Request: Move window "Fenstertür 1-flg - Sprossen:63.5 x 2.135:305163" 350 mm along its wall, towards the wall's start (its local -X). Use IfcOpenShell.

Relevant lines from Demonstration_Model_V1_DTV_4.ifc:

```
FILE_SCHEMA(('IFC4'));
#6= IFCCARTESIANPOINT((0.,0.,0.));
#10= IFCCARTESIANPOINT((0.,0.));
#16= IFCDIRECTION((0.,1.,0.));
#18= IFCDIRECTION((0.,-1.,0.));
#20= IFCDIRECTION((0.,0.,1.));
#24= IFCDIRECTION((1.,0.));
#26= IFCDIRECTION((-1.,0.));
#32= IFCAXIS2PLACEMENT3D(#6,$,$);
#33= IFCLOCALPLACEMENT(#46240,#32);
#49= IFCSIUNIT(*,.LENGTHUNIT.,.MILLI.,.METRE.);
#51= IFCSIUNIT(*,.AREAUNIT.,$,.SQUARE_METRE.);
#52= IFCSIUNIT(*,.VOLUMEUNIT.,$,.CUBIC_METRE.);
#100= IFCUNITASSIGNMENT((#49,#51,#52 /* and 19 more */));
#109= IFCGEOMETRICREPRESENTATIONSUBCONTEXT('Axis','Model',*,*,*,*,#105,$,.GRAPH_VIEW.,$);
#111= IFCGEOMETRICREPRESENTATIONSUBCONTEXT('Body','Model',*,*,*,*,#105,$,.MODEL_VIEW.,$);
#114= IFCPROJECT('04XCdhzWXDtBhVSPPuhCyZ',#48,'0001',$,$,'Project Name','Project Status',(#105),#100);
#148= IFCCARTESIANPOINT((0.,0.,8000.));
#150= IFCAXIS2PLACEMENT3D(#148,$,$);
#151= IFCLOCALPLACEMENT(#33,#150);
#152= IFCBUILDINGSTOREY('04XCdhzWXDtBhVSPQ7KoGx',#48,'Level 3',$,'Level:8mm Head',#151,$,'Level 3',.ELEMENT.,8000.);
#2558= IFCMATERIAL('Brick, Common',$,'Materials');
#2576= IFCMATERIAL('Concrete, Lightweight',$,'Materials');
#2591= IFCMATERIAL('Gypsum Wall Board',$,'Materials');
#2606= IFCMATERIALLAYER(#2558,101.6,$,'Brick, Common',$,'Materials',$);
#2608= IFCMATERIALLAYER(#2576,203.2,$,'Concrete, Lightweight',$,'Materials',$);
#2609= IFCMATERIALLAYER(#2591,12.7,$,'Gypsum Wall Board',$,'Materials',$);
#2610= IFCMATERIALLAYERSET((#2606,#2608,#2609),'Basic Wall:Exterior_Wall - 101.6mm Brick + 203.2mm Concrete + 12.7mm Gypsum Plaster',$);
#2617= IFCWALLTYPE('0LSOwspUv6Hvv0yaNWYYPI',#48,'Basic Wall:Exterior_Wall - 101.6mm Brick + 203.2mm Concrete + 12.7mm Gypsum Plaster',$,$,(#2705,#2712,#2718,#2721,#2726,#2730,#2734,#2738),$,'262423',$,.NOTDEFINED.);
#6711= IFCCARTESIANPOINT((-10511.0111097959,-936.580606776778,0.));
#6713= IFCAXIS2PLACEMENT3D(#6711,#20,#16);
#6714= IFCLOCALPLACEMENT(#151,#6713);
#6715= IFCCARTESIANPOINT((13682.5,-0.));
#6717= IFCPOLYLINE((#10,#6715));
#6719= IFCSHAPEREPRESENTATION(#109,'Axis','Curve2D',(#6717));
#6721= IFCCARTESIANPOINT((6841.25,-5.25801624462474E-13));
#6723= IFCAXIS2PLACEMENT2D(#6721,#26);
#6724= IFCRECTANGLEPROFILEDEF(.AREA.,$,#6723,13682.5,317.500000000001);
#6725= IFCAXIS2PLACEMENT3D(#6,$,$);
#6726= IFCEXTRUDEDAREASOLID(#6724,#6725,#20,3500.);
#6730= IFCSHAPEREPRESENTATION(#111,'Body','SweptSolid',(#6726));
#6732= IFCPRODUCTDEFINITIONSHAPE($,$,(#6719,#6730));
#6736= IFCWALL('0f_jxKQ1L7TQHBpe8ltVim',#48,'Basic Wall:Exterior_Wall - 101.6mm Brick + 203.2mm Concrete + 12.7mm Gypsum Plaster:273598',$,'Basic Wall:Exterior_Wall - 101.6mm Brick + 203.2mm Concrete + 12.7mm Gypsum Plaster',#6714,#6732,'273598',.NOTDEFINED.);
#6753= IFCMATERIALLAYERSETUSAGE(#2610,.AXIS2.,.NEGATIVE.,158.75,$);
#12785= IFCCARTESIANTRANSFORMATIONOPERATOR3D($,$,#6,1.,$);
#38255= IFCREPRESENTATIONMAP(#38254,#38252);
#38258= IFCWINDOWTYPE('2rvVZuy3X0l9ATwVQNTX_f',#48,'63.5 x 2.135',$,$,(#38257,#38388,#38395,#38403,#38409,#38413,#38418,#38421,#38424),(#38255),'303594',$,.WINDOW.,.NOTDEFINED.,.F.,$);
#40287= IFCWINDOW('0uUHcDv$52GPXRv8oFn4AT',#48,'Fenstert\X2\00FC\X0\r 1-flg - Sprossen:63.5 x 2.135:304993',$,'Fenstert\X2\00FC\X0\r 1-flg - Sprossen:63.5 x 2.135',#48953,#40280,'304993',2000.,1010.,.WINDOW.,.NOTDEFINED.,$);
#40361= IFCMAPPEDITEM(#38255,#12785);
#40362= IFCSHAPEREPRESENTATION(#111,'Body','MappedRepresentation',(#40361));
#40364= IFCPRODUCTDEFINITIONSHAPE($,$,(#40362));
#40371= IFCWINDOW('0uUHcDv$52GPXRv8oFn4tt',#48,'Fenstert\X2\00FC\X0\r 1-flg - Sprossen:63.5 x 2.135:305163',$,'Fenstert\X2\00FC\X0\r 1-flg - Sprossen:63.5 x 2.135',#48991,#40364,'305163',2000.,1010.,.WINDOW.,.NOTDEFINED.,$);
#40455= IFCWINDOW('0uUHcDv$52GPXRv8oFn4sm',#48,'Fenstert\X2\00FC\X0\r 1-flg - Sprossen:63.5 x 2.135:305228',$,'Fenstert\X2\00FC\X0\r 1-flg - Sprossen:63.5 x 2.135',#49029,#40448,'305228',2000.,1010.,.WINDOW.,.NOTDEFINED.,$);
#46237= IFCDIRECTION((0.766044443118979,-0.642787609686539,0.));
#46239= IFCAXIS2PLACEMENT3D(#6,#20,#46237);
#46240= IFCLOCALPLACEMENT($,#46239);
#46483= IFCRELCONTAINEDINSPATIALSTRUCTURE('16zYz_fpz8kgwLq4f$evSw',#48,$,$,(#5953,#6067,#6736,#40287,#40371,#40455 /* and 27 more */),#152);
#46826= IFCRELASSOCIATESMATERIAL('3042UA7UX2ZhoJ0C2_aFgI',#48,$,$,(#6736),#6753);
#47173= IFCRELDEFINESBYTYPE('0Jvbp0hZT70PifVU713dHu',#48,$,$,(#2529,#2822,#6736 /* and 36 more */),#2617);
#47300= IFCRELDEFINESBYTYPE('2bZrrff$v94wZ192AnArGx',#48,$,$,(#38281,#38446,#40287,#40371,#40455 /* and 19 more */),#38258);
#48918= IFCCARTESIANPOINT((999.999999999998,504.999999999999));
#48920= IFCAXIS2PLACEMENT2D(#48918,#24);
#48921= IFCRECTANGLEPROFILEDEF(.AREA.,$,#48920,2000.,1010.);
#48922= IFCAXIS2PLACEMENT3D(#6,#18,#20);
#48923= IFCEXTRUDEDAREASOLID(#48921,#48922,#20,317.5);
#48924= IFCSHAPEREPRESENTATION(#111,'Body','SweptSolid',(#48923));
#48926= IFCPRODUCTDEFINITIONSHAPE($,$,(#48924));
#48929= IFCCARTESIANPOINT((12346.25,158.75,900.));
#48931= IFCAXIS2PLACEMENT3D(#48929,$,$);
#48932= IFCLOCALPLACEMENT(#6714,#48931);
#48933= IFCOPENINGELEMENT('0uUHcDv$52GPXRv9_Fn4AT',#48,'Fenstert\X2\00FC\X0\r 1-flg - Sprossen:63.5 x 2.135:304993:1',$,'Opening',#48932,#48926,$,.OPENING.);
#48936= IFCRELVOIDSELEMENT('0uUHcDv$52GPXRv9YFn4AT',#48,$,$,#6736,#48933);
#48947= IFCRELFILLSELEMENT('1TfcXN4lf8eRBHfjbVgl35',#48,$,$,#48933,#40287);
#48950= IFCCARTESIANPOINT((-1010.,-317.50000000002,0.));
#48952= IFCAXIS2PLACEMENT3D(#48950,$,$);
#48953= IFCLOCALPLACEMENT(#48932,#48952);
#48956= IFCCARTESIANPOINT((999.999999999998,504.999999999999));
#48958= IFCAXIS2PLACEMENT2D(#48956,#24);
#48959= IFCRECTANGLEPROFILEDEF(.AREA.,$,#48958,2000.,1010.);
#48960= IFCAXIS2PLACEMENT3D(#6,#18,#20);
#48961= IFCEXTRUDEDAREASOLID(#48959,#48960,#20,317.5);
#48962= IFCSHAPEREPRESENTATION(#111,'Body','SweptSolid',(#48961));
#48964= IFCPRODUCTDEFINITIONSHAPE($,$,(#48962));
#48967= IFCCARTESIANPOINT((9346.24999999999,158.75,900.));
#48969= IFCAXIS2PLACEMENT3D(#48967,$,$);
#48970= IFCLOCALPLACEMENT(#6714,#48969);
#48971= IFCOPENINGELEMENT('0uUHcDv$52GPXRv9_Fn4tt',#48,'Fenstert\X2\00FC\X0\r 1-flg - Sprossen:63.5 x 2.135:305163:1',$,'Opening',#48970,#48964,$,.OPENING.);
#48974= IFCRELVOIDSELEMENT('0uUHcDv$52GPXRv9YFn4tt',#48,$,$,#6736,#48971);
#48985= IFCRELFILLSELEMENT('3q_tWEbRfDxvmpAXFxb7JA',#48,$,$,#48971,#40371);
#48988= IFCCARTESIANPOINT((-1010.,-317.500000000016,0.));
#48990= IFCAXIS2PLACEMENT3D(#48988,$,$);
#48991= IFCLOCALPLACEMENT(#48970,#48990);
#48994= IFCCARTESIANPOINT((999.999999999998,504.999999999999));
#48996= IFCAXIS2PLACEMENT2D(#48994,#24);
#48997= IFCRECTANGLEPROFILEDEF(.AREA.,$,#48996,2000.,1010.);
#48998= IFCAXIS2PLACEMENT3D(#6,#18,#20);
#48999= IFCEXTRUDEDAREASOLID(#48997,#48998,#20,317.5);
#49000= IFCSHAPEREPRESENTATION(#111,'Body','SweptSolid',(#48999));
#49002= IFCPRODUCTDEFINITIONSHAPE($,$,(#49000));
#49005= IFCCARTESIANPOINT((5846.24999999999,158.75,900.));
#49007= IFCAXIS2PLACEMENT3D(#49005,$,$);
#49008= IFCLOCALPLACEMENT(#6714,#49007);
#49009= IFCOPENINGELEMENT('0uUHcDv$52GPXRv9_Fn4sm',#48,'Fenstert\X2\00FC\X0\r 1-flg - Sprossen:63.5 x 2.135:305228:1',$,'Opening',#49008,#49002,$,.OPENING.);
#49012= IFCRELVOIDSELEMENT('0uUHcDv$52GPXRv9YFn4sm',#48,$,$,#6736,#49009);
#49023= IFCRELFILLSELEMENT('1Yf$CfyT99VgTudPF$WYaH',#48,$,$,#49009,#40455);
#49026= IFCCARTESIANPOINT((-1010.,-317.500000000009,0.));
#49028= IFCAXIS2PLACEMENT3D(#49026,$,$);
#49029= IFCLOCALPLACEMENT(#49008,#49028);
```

```python
import ifcopenshell
import ifcopenshell.api.geometry
import ifcopenshell.util.placement
import ifcopenshell.util.unit

model = ifcopenshell.open("Demonstration_Model_V1_DTV_4.ifc")
unit_scale = ifcopenshell.util.unit.calculate_unit_scale(model)

window = model.by_id(40371)
opening = window.FillsVoids[0].RelatingOpeningElement
wall = opening.VoidsElements[0].RelatingBuildingElement

wall_matrix = ifcopenshell.util.placement.get_local_placement(wall.ObjectPlacement)
shift = wall_matrix[:3, 0] * -0.35 / unit_scale
before = ifcopenshell.util.placement.get_local_placement(window.ObjectPlacement)[:3, 3].copy()

# The window is placed relative to its opening, so it follows when the opening moves.
matrix = ifcopenshell.util.placement.get_local_placement(opening.ObjectPlacement)
matrix[:3, 3] += shift
ifcopenshell.api.geometry.edit_object_placement(
    model, product=opening, matrix=matrix, is_si=False, should_transform_children=True
)

after = ifcopenshell.util.placement.get_local_placement(window.ObjectPlacement)[:3, 3]
print("window moved by", (after - before).round(3) + 0.0)

model.write("Demonstration_Model_V1_DTV_4_edited.ifc")
```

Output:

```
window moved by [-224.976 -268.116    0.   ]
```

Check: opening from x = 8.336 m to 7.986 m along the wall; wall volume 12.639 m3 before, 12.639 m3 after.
